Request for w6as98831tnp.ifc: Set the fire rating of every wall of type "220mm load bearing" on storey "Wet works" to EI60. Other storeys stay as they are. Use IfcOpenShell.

First a look at what the model holds.

```python
import ifcopenshell
import ifcopenshell.util.element

model = ifcopenshell.open("w6as98831tnp.ifc")
print(model.schema)
storey = next(s for s in model.by_type("IfcBuildingStorey") if s.Name == "Wet works")
walls = [e for e in ifcopenshell.util.element.get_decomposition(storey) if e.is_a("IfcWall")]
seen = {}
for e in walls:
    element_type = ifcopenshell.util.element.get_type(e)
    key = (element_type.Name if element_type != e and element_type else None, ifcopenshell.util.element.get_pset(e, "Pset_WallCommon", "FireRating"))
    seen[key] = seen.get(key, 0) + 1
for (name, value), count in sorted(seen.items(), key=str):
    print(count, "x", name, "|", value)
```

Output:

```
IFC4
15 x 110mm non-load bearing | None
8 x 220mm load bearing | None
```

```python
import ifcopenshell
import ifcopenshell.api.pset
import ifcopenshell.util.element

model = ifcopenshell.open("w6as98831tnp.ifc")

storey = next(s for s in model.by_type("IfcBuildingStorey") if s.Name == "Wet works")
walls = [e for e in ifcopenshell.util.element.get_decomposition(storey) if e.is_a("IfcWall")]

count = 0
for e in walls:
    element_type = ifcopenshell.util.element.get_type(e)
    if element_type in (None, e) or element_type.Name != "220mm load bearing":
        continue
    # add_pset returns the element's existing set when there is one.
    pset = ifcopenshell.api.pset.add_pset(model, product=e, name="Pset_WallCommon")
    ifcopenshell.api.pset.edit_pset(model, pset=pset, properties={"FireRating": "EI60"})
    count += 1

print(count, "walls updated")

model.write("w6as98831tnp-out.ifc")
```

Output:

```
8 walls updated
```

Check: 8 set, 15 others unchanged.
